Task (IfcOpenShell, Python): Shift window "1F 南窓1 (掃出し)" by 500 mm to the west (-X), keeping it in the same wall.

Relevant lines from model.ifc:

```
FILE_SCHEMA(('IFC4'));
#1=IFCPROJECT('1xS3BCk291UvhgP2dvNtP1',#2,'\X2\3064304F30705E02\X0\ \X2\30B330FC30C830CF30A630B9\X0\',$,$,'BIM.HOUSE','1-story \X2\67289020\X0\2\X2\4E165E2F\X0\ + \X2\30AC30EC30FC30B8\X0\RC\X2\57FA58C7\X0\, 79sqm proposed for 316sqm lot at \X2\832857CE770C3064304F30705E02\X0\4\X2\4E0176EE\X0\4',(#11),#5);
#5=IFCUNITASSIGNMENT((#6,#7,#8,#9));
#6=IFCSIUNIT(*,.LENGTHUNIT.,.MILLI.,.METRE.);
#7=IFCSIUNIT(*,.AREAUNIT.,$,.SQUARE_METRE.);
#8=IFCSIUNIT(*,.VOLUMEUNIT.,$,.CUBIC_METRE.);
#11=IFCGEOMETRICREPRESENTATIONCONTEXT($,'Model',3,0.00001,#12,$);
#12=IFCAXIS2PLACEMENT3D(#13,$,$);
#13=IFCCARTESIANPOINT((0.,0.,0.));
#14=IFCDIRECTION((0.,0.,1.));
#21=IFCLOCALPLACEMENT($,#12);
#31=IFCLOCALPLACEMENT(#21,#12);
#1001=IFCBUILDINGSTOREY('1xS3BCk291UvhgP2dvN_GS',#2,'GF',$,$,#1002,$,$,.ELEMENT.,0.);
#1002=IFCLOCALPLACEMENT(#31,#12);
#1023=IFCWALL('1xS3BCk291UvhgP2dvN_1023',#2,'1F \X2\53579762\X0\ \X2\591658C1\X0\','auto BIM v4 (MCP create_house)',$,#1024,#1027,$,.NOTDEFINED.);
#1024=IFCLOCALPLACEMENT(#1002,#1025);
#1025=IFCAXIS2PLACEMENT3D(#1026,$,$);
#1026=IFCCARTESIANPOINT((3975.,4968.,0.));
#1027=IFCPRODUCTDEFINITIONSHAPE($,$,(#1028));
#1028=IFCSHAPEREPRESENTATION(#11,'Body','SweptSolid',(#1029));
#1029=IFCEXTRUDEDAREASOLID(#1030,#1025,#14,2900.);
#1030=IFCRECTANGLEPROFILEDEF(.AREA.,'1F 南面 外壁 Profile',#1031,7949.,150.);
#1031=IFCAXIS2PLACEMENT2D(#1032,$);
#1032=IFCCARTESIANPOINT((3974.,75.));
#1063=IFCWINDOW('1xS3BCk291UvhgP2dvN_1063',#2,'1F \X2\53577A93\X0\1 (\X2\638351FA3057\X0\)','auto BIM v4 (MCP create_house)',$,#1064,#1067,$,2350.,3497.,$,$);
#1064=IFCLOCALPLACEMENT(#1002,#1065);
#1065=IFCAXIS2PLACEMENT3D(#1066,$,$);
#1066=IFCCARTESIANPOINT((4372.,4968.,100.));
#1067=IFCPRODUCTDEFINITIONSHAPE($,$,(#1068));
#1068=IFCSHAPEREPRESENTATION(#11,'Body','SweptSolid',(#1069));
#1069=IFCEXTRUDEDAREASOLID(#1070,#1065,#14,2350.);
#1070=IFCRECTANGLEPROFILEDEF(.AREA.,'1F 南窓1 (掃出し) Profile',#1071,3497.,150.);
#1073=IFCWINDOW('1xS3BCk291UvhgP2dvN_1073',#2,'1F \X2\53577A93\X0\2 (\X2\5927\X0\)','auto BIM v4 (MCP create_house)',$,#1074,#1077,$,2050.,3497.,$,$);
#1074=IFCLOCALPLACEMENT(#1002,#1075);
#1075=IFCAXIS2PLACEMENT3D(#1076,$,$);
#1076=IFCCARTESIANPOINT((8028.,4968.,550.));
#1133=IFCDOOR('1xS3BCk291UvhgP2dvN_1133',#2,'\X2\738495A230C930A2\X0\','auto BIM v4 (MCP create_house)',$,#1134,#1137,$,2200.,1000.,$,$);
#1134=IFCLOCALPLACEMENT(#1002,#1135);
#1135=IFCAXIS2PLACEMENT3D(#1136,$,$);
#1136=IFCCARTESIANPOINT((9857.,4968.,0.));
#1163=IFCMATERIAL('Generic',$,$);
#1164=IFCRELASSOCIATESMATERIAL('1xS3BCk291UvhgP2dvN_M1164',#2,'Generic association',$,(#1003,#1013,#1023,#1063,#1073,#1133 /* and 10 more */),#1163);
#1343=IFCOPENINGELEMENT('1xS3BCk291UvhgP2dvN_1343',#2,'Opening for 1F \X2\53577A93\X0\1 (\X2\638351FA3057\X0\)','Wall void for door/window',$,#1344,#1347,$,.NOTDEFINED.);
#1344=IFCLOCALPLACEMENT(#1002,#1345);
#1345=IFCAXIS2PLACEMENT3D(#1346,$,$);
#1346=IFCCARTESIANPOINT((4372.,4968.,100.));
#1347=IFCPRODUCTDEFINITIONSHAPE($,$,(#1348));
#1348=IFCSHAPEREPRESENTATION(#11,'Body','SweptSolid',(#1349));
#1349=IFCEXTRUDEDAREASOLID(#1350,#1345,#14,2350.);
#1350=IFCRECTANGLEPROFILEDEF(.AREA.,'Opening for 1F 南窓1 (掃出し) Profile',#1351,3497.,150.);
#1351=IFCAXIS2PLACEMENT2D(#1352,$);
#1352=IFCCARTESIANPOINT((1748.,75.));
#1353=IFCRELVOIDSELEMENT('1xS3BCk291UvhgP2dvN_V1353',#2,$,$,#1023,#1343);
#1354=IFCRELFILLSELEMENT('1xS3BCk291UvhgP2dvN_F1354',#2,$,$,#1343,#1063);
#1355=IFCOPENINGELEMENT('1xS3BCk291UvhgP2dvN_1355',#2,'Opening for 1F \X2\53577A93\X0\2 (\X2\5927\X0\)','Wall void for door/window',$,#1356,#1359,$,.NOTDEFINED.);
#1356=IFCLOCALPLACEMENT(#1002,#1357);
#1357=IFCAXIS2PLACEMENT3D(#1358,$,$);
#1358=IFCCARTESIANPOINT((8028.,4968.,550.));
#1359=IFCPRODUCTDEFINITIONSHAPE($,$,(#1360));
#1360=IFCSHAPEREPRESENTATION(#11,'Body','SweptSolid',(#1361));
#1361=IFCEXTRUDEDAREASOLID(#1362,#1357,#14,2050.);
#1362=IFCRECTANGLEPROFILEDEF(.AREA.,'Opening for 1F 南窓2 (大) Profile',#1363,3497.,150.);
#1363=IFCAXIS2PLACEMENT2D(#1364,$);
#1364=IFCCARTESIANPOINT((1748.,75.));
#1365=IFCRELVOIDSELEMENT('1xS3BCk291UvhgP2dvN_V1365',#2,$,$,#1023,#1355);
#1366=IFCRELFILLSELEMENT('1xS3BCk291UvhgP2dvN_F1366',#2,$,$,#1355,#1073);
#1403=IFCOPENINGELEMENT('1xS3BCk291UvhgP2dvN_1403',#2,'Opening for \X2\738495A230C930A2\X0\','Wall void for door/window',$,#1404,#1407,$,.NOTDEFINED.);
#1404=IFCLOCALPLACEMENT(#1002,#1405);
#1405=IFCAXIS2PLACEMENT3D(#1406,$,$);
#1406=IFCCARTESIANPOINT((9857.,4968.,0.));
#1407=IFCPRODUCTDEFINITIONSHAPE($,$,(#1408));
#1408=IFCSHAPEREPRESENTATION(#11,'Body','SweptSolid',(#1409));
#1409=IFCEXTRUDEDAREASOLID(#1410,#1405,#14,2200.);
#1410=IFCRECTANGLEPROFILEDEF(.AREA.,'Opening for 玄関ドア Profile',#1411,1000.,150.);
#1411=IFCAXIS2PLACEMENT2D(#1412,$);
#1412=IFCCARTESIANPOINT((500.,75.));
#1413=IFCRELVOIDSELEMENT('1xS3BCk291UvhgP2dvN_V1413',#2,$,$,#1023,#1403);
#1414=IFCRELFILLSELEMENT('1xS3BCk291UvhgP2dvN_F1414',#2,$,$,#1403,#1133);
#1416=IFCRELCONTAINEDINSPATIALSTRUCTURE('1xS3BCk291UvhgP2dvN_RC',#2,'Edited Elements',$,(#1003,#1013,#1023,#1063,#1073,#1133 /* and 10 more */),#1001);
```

```python
import ifcopenshell
import ifcopenshell.api.geometry
import ifcopenshell.util.placement
import ifcopenshell.util.unit

model = ifcopenshell.open("model.ifc")
unit_scale = ifcopenshell.util.unit.calculate_unit_scale(model)

window = model.by_guid("1xS3BCk291UvhgP2dvN_1063")
opening = window.FillsVoids[0].RelatingOpeningElement
wall = opening.VoidsElements[0].RelatingBuildingElement

wall_matrix = ifcopenshell.util.placement.get_local_placement(wall.ObjectPlacement)
shift = wall_matrix[:3, 0] * -0.5 / unit_scale
before = ifcopenshell.util.placement.get_local_placement(window.ObjectPlacement)[:3, 3].copy()

# The window is not placed relative to its opening, so move both.
for product in (opening, window):
    matrix = ifcopenshell.util.placement.get_local_placement(product.ObjectPlacement)
    matrix[:3, 3] += shift
    ifcopenshell.api.geometry.edit_object_placement(model, product=product, matrix=matrix, is_si=False)

after = ifcopenshell.util.placement.get_local_placement(window.ObjectPlacement)[:3, 3]
print("window moved by", (after - before).round(3) + 0.0)

model.write("model-out.ifc")
```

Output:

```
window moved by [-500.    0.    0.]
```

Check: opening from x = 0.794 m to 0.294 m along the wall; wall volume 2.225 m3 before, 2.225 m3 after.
